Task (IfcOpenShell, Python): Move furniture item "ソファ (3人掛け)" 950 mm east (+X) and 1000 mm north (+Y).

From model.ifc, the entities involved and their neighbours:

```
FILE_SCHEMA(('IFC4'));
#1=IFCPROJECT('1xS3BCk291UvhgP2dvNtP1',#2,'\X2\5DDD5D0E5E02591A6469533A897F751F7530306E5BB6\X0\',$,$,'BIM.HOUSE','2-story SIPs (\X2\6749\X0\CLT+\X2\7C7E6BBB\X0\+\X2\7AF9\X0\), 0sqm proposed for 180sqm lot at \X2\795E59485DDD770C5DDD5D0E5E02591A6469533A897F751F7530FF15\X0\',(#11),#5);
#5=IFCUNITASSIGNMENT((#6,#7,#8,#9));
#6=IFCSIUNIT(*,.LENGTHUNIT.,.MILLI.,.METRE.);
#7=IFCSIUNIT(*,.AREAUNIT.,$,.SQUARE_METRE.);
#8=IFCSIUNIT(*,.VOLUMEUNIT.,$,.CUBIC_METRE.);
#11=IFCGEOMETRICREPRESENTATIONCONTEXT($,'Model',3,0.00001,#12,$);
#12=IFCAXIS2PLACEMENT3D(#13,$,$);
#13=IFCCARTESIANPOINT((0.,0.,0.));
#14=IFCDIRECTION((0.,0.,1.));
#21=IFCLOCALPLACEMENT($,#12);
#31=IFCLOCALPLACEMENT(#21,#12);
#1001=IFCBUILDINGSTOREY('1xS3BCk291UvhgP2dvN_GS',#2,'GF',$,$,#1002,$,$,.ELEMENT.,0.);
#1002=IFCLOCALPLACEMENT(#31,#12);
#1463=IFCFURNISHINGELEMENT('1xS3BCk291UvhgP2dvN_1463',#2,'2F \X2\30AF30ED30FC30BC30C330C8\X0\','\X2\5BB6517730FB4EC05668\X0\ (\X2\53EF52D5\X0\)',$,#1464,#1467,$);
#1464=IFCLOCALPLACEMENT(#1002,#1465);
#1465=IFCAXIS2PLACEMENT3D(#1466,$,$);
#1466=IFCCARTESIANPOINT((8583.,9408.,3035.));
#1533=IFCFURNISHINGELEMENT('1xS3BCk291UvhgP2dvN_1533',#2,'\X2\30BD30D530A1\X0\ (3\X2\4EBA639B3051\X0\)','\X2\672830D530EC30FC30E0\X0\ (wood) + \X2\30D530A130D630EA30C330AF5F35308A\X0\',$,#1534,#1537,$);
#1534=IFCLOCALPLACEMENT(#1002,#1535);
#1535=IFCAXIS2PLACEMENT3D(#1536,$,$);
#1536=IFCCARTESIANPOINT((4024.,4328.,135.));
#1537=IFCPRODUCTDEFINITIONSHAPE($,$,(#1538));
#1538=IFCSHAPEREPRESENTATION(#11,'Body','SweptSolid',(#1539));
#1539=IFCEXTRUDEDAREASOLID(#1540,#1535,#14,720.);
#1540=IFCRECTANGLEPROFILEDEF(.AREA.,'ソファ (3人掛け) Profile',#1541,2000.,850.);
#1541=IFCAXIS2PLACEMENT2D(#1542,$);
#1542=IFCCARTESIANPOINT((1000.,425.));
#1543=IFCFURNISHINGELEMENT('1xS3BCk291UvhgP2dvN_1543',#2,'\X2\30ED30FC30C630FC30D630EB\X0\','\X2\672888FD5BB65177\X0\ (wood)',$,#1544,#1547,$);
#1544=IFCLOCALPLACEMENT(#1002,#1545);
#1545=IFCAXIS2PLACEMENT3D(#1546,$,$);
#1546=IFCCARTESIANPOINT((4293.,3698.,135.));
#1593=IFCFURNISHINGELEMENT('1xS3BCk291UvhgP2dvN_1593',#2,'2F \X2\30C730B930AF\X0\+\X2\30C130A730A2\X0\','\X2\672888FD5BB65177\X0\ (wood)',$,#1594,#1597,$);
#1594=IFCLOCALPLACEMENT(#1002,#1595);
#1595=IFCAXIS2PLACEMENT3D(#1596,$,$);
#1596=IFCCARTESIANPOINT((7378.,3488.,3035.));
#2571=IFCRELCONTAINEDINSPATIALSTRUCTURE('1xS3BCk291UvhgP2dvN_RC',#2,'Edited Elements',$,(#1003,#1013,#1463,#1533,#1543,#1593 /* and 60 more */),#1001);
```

```python
import ifcopenshell
import ifcopenshell.api.geometry
import ifcopenshell.util.placement
import ifcopenshell.util.unit

model = ifcopenshell.open("model.ifc")
unit_scale = ifcopenshell.util.unit.calculate_unit_scale(model)

item = model.by_guid("1xS3BCk291UvhgP2dvN_1533")
matrix = ifcopenshell.util.placement.get_local_placement(item.ObjectPlacement)
matrix[0, 3] += 0.95 / unit_scale
matrix[1, 3] += 1 / unit_scale
ifcopenshell.api.geometry.edit_object_placement(model, product=item, matrix=matrix, is_si=False)

print(ifcopenshell.util.placement.get_local_placement(item.ObjectPlacement).round(3) + 0.0)

model.write("model_rev.ifc")
```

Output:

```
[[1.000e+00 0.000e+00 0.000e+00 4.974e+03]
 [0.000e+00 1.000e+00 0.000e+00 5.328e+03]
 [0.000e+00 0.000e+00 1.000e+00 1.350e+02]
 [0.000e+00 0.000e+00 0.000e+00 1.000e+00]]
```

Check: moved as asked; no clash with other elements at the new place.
